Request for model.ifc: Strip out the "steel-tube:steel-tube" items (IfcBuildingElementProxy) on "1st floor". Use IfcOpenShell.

First a look at what the model holds.

```python
import ifcopenshell
import ifcopenshell.util.element

model = ifcopenshell.open("model.ifc")
print(model.schema)
storey = next(s for s in model.by_type("IfcBuildingStorey") if s.Name == "1st floor")
proxies = [e for e in ifcopenshell.util.element.get_decomposition(storey) if e.is_a("IfcBuildingElementProxy")]
seen = {}
for e in proxies:
    element_type = ifcopenshell.util.element.get_type(e)
    name = element_type.Name if element_type not in (None, e) else None
    seen[name] = seen.get(name, 0) + 1
for name, count in sorted(seen.items(), key=str):
    print(count, "x", name)
```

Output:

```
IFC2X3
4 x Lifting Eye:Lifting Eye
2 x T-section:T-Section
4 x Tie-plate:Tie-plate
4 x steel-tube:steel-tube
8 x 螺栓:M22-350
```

```python
import ifcopenshell
import ifcopenshell.api.root
import ifcopenshell.util.element

model = ifcopenshell.open("model.ifc")

storey = next(s for s in model.by_type("IfcBuildingStorey") if s.Name == "1st floor")
proxies = [e for e in ifcopenshell.util.element.get_decomposition(storey) if e.is_a("IfcBuildingElementProxy")]
targets = [e for e in proxies if (t := ifcopenshell.util.element.get_type(e)) not in (None, e) and t.Name == "steel-tube:steel-tube"]

for e in targets:
    ifcopenshell.api.root.remove_product(model, product=e)
print(len(targets), "removed")

model.write("model_v2.ifc")
```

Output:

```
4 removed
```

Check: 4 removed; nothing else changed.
